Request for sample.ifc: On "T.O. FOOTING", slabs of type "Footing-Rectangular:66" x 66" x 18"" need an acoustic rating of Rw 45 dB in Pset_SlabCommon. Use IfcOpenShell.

First a look at what the model holds.

```python
import ifcopenshell
import ifcopenshell.util.element

model = ifcopenshell.open("sample.ifc")
print(model.schema)
storey = next(s for s in model.by_type("IfcBuildingStorey") if s.Name == "T.O. FOOTING")
slabs = [e for e in ifcopenshell.util.element.get_decomposition(storey) if e.is_a("IfcSlab")]
seen = {}
for e in slabs:
    element_type = ifcopenshell.util.element.get_type(e)
    key = (element_type.Name if element_type != e and element_type else None, ifcopenshell.util.element.get_pset(e, "Pset_SlabCommon", "AcousticRating"))
    seen[key] = seen.get(key, 0) + 1
for (name, value), count in sorted(seen.items(), key=str):
    print(count, "x", name, "|", value)
```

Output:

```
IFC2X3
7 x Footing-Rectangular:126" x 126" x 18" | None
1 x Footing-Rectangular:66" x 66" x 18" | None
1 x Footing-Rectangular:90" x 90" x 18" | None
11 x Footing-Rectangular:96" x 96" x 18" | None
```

```python
import ifcopenshell
import ifcopenshell.api.pset
import ifcopenshell.util.element

model = ifcopenshell.open("sample.ifc")

storey = next(s for s in model.by_type("IfcBuildingStorey") if s.Name == "T.O. FOOTING")
slabs = [e for e in ifcopenshell.util.element.get_decomposition(storey) if e.is_a("IfcSlab")]

count = 0
for e in slabs:
    element_type = ifcopenshell.util.element.get_type(e)
    if element_type in (None, e) or element_type.Name != 'Footing-Rectangular:66" x 66" x 18"':
        continue
    # add_pset returns the element's existing set when there is one.
    pset = ifcopenshell.api.pset.add_pset(model, product=e, name="Pset_SlabCommon")
    ifcopenshell.api.pset.edit_pset(model, pset=pset, properties={"AcousticRating": "Rw 45 dB"})
    count += 1

print(count, "slabs updated")

model.write("sample-out.ifc")
```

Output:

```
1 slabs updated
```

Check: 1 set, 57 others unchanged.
